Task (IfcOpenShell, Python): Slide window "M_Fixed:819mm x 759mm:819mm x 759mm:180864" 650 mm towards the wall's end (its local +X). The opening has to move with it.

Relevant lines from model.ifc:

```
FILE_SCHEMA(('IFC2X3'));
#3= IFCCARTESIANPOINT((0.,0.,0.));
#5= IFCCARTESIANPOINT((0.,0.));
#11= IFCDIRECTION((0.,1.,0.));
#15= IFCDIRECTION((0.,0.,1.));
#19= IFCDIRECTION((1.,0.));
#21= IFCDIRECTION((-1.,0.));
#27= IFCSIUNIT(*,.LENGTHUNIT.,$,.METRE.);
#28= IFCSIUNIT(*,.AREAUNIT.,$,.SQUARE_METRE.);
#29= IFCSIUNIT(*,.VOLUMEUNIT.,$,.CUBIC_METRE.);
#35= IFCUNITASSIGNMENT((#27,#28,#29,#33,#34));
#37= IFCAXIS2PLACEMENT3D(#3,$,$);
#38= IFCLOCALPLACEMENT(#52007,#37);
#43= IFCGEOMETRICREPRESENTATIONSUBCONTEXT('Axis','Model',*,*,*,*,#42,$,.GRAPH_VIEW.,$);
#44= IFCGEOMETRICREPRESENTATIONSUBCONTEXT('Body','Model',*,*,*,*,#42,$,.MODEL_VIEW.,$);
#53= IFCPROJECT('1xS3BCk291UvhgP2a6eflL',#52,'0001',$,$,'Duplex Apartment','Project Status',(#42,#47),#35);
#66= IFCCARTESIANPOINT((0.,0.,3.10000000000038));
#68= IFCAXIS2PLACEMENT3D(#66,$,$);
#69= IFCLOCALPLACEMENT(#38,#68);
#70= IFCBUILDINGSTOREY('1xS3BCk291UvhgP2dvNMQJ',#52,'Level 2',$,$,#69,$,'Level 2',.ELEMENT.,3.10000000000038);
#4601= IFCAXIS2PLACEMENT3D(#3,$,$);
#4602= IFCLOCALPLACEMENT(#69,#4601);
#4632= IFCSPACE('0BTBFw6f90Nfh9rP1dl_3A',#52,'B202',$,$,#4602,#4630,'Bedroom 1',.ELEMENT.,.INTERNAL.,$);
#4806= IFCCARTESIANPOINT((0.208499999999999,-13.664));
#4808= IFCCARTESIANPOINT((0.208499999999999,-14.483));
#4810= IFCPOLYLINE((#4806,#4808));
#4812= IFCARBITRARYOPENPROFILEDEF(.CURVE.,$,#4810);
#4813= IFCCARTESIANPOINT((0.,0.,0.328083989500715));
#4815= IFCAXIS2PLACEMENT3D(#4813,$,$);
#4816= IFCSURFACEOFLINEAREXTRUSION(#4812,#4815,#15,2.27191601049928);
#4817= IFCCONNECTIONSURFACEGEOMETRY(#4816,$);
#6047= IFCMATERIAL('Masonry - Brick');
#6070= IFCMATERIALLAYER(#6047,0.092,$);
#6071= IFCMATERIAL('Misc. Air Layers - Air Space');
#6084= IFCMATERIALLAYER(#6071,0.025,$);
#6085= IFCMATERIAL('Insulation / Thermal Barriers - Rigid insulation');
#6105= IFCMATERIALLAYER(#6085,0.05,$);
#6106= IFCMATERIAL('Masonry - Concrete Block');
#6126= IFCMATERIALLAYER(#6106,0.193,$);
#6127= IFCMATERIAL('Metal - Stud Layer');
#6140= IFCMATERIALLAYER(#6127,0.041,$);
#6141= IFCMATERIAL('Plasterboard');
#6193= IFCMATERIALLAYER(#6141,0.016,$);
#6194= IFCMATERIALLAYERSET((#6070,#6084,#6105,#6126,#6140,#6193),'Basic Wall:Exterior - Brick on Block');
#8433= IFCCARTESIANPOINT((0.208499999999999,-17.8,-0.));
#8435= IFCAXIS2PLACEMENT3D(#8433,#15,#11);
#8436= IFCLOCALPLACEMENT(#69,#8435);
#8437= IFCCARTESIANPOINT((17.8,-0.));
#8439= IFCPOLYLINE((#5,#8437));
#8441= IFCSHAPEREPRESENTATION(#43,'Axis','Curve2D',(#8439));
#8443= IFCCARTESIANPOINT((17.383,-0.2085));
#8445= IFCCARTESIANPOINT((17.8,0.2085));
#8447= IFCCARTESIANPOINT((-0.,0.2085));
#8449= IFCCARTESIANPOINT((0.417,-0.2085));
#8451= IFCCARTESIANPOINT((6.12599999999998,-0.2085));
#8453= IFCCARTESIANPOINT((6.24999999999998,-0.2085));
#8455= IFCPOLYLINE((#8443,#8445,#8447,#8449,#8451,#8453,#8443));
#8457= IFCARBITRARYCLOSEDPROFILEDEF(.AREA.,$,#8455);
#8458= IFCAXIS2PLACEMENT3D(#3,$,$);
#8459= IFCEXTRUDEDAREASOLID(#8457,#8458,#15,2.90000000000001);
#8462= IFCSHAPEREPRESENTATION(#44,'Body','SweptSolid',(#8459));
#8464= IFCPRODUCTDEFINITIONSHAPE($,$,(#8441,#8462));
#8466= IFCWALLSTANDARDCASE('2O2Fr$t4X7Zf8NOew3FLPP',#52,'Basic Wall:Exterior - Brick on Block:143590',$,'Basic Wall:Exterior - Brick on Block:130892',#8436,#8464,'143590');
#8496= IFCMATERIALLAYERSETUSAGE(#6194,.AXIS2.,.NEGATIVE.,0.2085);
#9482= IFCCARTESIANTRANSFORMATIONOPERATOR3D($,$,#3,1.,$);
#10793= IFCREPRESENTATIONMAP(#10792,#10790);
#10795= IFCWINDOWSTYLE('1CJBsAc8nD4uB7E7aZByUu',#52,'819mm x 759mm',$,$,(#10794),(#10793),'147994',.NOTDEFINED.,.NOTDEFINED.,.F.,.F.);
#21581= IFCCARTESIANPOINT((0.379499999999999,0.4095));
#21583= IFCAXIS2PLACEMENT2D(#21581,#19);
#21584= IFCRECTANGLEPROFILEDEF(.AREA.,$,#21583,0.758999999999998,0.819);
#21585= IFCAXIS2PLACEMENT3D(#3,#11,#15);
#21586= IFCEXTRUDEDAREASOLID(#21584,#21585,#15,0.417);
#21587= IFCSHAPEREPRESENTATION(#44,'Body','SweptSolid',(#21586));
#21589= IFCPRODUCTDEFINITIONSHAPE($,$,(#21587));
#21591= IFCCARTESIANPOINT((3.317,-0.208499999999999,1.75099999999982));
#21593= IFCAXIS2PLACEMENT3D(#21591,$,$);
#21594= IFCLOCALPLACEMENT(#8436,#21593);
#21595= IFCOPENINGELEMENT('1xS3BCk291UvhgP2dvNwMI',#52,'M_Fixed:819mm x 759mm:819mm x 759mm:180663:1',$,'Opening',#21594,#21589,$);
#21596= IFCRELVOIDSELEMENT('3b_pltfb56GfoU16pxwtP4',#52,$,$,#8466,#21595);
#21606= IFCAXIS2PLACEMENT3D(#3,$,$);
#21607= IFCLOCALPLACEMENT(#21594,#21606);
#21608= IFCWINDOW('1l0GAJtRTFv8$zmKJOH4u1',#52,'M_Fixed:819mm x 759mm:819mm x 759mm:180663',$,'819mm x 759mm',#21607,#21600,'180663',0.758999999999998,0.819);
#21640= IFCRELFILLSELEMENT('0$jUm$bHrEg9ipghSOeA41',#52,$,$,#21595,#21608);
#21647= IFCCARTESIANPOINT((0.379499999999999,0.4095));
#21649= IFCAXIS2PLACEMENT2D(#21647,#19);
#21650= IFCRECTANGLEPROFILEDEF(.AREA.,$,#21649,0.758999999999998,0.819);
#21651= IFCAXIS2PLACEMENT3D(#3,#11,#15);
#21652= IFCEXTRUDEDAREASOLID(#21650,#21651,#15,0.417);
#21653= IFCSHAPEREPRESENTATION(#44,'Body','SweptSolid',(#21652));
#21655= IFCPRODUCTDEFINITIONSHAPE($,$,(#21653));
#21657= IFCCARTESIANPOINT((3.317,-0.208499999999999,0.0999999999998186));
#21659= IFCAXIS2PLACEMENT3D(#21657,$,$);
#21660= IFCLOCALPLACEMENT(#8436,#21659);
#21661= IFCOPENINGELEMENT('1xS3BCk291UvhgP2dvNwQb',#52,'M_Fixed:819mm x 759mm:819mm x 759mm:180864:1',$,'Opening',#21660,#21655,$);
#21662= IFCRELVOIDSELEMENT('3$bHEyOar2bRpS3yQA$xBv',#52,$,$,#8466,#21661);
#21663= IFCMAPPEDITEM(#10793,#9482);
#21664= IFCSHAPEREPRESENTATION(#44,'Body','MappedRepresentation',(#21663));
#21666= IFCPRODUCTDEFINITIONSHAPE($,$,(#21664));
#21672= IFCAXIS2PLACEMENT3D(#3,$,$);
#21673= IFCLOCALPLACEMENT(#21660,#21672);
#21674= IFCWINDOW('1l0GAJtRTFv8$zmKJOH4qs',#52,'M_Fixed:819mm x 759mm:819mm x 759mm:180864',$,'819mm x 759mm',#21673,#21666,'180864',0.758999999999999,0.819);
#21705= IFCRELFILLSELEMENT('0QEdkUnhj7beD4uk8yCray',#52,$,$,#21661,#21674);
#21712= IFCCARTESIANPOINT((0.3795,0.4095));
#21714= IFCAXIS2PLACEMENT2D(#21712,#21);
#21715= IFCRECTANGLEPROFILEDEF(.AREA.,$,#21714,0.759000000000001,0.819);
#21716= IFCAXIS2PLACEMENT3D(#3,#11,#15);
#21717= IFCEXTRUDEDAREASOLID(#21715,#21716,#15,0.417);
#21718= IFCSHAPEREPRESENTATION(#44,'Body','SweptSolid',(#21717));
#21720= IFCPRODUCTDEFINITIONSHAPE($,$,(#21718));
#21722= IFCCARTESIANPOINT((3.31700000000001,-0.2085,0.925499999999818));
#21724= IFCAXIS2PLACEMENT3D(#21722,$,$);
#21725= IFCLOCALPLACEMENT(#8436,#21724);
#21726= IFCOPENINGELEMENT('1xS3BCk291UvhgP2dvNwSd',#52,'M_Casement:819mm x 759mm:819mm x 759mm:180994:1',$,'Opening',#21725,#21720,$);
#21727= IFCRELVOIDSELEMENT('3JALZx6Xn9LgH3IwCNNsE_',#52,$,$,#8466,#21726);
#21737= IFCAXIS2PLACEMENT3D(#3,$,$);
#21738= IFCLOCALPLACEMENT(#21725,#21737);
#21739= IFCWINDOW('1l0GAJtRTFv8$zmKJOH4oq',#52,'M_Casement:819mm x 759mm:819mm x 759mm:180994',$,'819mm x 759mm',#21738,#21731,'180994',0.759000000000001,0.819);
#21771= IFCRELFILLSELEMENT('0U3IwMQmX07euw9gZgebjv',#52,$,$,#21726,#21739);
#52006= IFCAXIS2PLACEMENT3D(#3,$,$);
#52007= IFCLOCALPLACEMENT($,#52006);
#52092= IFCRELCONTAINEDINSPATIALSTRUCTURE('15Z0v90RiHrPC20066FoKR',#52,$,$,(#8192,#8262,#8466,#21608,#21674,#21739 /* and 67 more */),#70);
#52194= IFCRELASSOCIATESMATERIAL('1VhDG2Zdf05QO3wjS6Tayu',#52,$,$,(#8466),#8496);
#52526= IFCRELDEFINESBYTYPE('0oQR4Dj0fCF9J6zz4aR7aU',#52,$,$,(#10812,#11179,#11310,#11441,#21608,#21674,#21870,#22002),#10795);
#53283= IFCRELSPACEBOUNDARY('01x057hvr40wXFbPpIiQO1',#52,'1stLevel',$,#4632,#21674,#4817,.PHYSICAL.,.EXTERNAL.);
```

```python
import numpy as np
import ifcopenshell
import ifcopenshell.api.geometry
import ifcopenshell.util.placement

model = ifcopenshell.open("model.ifc")

window = model.by_guid("1l0GAJtRTFv8$zmKJOH4qs")
opening = window.FillsVoids[0].RelatingOpeningElement
wall = opening.VoidsElements[0].RelatingBuildingElement

wall_matrix = ifcopenshell.util.placement.get_local_placement(wall.ObjectPlacement)
shift = wall_matrix[:3, 0] * 0.65
before = ifcopenshell.util.placement.get_local_placement(window.ObjectPlacement)[:3, 3].copy()

# The window is placed relative to its opening, so it follows when the opening moves.
matrix = ifcopenshell.util.placement.get_local_placement(opening.ObjectPlacement)
matrix[:3, 3] += shift
ifcopenshell.api.geometry.edit_object_placement(
    model, product=opening, matrix=matrix, is_si=False, should_transform_children=True
)

# Space boundary surfaces are stored in each space's coordinates; move them too.
for rel in window.ProvidesBoundaries:
    if not rel.ConnectionGeometry:
        continue
    surface = rel.ConnectionGeometry.SurfaceOnRelatingElement
    space_matrix = ifcopenshell.util.placement.get_local_placement(rel.RelatingSpace.ObjectPlacement)
    point = np.array(surface.Position.Location.Coordinates) + space_matrix[:3, :3].T @ shift
    surface.Position = model.createIfcAxis2Placement3D(
        model.createIfcCartesianPoint(point.tolist()), surface.Position.Axis, surface.Position.RefDirection
    )

after = ifcopenshell.util.placement.get_local_placement(window.ObjectPlacement)[:3, 3]
print("window moved by", (after - before).round(3) + 0.0)

model.write("model-out.ifc")
```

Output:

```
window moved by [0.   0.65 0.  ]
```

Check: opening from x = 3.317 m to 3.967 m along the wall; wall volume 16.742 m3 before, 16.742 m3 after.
